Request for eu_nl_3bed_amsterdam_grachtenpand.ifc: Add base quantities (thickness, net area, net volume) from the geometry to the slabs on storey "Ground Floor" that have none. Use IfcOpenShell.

First a look at what the model holds.

```python
import ifcopenshell
import ifcopenshell.util.element
import ifcopenshell.util.unit

model = ifcopenshell.open("eu_nl_3bed_amsterdam_grachtenpand.ifc")
print(model.schema)
for unit_type in ("LENGTHUNIT", "AREAUNIT", "VOLUMEUNIT"):
    print(unit_type, ifcopenshell.util.unit.calculate_unit_scale(model, unit_type))
storey = next(s for s in model.by_type("IfcBuildingStorey") if s.Name == "Ground Floor")
slabs = [e for e in ifcopenshell.util.element.get_decomposition(storey) if e.is_a("IfcSlab")]
for e in sorted(slabs, key=lambda e: e.id()):
    print(e.id(), e.is_a(), e.Name, list(ifcopenshell.util.element.get_psets(e, qtos_only=True)), sep=" | ")
```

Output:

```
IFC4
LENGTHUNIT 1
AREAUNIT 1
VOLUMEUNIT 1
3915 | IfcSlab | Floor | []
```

```python
import ifcopenshell
import ifcopenshell.api.pset
import ifcopenshell.geom
import ifcopenshell.util.element
import ifcopenshell.util.shape
import ifcopenshell.util.unit

model = ifcopenshell.open("eu_nl_3bed_amsterdam_grachtenpand.ifc")
unit_scale = ifcopenshell.util.unit.calculate_unit_scale(model)
area_scale = ifcopenshell.util.unit.calculate_unit_scale(model, "AREAUNIT")
volume_scale = ifcopenshell.util.unit.calculate_unit_scale(model, "VOLUMEUNIT")
settings = ifcopenshell.geom.settings()

storey = next(s for s in model.by_type("IfcBuildingStorey") if s.Name == "Ground Floor")
slabs = [e for e in ifcopenshell.util.element.get_decomposition(storey) if e.is_a("IfcSlab")]

for e in sorted(slabs, key=lambda e: e.id()):
    if ifcopenshell.util.element.get_psets(e, qtos_only=True, should_inherit=False):
        continue
    # Geometry comes back in metres, in the element's own axes.
    shape = ifcopenshell.geom.create_shape(settings, e)
    values = {
        "Width": ifcopenshell.util.shape.get_z(shape.geometry) / unit_scale,
        "NetArea": ifcopenshell.util.shape.get_footprint_area(shape.geometry) / area_scale,
        "NetVolume": ifcopenshell.util.shape.get_volume(shape.geometry) / volume_scale,
    }
    qto = ifcopenshell.api.pset.add_qto(model, product=e, name="Qto_SlabBaseQuantities")
    ifcopenshell.api.pset.edit_qto(model, qto=qto, properties=values)
    print(e.id(), {k: round(v, 3) for k, v in values.items()})

model.write("eu_nl_3bed_amsterdam_grachtenpand_updated.ifc")
```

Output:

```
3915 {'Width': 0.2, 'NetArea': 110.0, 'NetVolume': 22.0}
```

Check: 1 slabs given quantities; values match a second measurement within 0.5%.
